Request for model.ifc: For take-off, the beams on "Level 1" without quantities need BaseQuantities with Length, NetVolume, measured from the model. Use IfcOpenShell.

First a look at what the model holds.

```python
import ifcopenshell
import ifcopenshell.util.element
import ifcopenshell.util.unit

model = ifcopenshell.open("model.ifc")
print(model.schema)
for unit_type in ("LENGTHUNIT", "AREAUNIT", "VOLUMEUNIT"):
    print(unit_type, ifcopenshell.util.unit.calculate_unit_scale(model, unit_type))
storey = next(s for s in model.by_type("IfcBuildingStorey") if s.Name == "Level 1")
beams = [e for e in ifcopenshell.util.element.get_decomposition(storey) if e.is_a("IfcBeam")]
for e in sorted(beams, key=lambda e: e.id()):
    print(e.id(), e.is_a(), e.Name, list(ifcopenshell.util.element.get_psets(e, qtos_only=True)), sep=" | ")
```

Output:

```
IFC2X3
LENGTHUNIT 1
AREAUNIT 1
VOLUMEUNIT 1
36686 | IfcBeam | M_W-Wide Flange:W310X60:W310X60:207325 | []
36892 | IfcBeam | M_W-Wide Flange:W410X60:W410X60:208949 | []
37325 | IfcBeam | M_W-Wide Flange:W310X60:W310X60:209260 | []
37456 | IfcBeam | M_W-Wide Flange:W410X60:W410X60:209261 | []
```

```python
import ifcopenshell
import ifcopenshell.api.pset
import ifcopenshell.geom
import ifcopenshell.util.element
import ifcopenshell.util.shape
import ifcopenshell.util.unit

model = ifcopenshell.open("model.ifc")
unit_scale = ifcopenshell.util.unit.calculate_unit_scale(model)
volume_scale = ifcopenshell.util.unit.calculate_unit_scale(model, "VOLUMEUNIT")
settings = ifcopenshell.geom.settings()

storey = next(s for s in model.by_type("IfcBuildingStorey") if s.Name == "Level 1")
beams = [e for e in ifcopenshell.util.element.get_decomposition(storey) if e.is_a("IfcBeam")]

for e in sorted(beams, key=lambda e: e.id()):
    if ifcopenshell.util.element.get_psets(e, qtos_only=True, should_inherit=False):
        continue
    # Geometry comes back in metres, in the element's own axes.
    shape = ifcopenshell.geom.create_shape(settings, e)
    values = {
        "Length": ifcopenshell.util.shape.get_max_xyz(shape.geometry) / unit_scale,
        "NetVolume": ifcopenshell.util.shape.get_volume(shape.geometry) / volume_scale,
    }
    qto = ifcopenshell.api.pset.add_qto(model, product=e, name="BaseQuantities")
    ifcopenshell.api.pset.edit_qto(model, qto=qto, properties=values)
    print(e.id(), {k: round(v, 3) for k, v in values.items()})

model.write("model_edited.ifc")
```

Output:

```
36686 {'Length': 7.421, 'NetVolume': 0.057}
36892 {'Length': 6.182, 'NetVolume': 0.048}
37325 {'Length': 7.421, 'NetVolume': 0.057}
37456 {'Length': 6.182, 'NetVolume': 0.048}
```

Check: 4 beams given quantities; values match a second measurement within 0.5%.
